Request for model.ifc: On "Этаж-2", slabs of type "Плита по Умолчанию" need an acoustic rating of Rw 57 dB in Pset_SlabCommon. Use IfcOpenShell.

First a look at what the model holds.

```python
import ifcopenshell
import ifcopenshell.util.element

model = ifcopenshell.open("model.ifc")
print(model.schema)
storey = next(s for s in model.by_type("IfcBuildingStorey") if s.Name == "Этаж-2")
slabs = [e for e in ifcopenshell.util.element.get_decomposition(storey) if e.is_a("IfcSlab")]
seen = {}
for e in slabs:
    element_type = ifcopenshell.util.element.get_type(e)
    key = (element_type.Name if element_type != e and element_type else None, ifcopenshell.util.element.get_pset(e, "Pset_SlabCommon", "AcousticRating"))
    seen[key] = seen.get(key, 0) + 1
for (name, value), count in sorted(seen.items(), key=str):
    print(count, "x", name, "|", value)
```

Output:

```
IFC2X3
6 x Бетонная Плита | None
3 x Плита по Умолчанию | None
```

```python
import ifcopenshell
import ifcopenshell.api.pset
import ifcopenshell.util.element

model = ifcopenshell.open("model.ifc")

storey = next(s for s in model.by_type("IfcBuildingStorey") if s.Name == "Этаж-2")
slabs = [e for e in ifcopenshell.util.element.get_decomposition(storey) if e.is_a("IfcSlab")]

count = 0
for e in slabs:
    element_type = ifcopenshell.util.element.get_type(e)
    if element_type in (None, e) or element_type.Name != "Плита по Умолчанию":
        continue
    # add_pset returns the element's existing set when there is one.
    pset = ifcopenshell.api.pset.add_pset(model, product=e, name="Pset_SlabCommon")
    ifcopenshell.api.pset.edit_pset(model, pset=pset, properties={"AcousticRating": "Rw 57 dB"})
    count += 1

print(count, "slabs updated")

model.write("model_v2.ifc")
```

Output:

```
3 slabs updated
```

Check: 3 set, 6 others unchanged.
